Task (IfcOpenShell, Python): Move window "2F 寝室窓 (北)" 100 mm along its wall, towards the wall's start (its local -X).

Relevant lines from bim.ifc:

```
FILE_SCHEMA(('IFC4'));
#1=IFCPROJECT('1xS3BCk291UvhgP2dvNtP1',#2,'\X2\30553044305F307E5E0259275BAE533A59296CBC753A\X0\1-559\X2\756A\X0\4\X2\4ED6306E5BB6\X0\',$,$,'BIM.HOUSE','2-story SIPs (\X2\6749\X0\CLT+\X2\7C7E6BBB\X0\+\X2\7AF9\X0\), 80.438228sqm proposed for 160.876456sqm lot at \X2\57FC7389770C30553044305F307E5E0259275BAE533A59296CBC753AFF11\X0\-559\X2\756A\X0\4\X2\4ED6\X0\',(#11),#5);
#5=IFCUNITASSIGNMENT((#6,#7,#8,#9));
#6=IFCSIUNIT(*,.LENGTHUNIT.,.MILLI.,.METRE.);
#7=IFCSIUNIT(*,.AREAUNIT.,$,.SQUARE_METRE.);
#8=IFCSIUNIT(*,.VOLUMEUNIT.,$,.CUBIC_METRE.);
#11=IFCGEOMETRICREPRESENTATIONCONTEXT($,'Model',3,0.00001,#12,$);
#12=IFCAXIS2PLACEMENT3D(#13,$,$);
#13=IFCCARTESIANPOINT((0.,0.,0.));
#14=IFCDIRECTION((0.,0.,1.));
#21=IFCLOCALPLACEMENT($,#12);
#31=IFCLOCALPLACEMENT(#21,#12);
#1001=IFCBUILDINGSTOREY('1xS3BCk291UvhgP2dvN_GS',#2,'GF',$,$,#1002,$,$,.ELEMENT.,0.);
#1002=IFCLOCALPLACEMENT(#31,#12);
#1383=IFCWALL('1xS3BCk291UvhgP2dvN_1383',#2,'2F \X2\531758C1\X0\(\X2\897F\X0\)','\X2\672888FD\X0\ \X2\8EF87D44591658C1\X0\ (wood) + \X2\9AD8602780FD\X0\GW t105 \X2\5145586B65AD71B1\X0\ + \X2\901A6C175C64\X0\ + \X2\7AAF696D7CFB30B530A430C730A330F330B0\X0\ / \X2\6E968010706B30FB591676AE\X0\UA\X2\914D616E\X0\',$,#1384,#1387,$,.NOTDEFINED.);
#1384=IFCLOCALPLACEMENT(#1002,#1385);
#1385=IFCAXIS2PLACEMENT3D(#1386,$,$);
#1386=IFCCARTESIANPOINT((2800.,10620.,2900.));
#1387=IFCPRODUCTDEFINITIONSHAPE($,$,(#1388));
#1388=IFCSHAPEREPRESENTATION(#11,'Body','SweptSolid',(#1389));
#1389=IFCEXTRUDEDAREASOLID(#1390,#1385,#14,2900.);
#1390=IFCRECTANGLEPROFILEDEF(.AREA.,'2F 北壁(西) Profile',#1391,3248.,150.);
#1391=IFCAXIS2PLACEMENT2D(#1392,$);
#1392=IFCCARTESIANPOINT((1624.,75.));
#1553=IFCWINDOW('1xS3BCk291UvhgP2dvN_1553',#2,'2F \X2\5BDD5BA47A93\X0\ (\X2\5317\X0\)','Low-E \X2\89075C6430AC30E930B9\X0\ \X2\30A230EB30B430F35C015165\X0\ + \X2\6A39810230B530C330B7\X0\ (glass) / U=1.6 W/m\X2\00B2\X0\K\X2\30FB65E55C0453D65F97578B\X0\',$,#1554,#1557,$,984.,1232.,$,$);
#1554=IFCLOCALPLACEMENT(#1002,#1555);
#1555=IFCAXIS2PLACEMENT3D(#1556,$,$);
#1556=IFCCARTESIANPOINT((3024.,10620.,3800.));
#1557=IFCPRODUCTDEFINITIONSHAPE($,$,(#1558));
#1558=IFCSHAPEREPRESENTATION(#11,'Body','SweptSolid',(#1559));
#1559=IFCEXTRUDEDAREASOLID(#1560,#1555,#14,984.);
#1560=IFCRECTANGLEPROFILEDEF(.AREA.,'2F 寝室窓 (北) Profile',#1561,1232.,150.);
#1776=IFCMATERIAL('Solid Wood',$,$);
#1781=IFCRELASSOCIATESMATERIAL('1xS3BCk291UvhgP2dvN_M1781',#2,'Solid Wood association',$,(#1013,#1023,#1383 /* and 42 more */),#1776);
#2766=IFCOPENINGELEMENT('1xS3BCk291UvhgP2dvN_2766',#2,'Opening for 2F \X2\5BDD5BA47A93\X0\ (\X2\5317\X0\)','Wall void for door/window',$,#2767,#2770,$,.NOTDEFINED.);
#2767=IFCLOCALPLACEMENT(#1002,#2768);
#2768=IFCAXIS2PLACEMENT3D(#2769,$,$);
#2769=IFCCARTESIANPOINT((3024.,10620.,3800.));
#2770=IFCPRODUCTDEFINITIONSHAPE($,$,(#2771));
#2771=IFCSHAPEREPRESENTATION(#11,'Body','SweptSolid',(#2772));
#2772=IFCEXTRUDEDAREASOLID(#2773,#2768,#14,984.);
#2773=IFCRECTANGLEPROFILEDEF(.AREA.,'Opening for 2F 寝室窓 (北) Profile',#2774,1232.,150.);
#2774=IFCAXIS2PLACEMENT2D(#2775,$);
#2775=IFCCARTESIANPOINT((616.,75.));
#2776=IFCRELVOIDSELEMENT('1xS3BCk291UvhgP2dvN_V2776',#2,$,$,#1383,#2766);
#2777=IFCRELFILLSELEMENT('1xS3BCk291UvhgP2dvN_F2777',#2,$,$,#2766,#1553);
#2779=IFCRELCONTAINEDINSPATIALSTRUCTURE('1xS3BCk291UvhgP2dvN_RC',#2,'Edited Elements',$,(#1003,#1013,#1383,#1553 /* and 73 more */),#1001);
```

```python
import ifcopenshell
import ifcopenshell.api.geometry
import ifcopenshell.util.placement
import ifcopenshell.util.unit

model = ifcopenshell.open("bim.ifc")
unit_scale = ifcopenshell.util.unit.calculate_unit_scale(model)

window = model.by_guid("1xS3BCk291UvhgP2dvN_1553")
opening = window.FillsVoids[0].RelatingOpeningElement
wall = opening.VoidsElements[0].RelatingBuildingElement

wall_matrix = ifcopenshell.util.placement.get_local_placement(wall.ObjectPlacement)
shift = wall_matrix[:3, 0] * -0.1 / unit_scale
before = ifcopenshell.util.placement.get_local_placement(window.ObjectPlacement)[:3, 3].copy()

# The window is not placed relative to its opening, so move both.
for product in (opening, window):
    matrix = ifcopenshell.util.placement.get_local_placement(product.ObjectPlacement)
    matrix[:3, 3] += shift
    ifcopenshell.api.geometry.edit_object_placement(model, product=product, matrix=matrix, is_si=False)

after = ifcopenshell.util.placement.get_local_placement(window.ObjectPlacement)[:3, 3]
print("window moved by", (after - before).round(3) + 0.0)

model.write("bim_v2.ifc")
```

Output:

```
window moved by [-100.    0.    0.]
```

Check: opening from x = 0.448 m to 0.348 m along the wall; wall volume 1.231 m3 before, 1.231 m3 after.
